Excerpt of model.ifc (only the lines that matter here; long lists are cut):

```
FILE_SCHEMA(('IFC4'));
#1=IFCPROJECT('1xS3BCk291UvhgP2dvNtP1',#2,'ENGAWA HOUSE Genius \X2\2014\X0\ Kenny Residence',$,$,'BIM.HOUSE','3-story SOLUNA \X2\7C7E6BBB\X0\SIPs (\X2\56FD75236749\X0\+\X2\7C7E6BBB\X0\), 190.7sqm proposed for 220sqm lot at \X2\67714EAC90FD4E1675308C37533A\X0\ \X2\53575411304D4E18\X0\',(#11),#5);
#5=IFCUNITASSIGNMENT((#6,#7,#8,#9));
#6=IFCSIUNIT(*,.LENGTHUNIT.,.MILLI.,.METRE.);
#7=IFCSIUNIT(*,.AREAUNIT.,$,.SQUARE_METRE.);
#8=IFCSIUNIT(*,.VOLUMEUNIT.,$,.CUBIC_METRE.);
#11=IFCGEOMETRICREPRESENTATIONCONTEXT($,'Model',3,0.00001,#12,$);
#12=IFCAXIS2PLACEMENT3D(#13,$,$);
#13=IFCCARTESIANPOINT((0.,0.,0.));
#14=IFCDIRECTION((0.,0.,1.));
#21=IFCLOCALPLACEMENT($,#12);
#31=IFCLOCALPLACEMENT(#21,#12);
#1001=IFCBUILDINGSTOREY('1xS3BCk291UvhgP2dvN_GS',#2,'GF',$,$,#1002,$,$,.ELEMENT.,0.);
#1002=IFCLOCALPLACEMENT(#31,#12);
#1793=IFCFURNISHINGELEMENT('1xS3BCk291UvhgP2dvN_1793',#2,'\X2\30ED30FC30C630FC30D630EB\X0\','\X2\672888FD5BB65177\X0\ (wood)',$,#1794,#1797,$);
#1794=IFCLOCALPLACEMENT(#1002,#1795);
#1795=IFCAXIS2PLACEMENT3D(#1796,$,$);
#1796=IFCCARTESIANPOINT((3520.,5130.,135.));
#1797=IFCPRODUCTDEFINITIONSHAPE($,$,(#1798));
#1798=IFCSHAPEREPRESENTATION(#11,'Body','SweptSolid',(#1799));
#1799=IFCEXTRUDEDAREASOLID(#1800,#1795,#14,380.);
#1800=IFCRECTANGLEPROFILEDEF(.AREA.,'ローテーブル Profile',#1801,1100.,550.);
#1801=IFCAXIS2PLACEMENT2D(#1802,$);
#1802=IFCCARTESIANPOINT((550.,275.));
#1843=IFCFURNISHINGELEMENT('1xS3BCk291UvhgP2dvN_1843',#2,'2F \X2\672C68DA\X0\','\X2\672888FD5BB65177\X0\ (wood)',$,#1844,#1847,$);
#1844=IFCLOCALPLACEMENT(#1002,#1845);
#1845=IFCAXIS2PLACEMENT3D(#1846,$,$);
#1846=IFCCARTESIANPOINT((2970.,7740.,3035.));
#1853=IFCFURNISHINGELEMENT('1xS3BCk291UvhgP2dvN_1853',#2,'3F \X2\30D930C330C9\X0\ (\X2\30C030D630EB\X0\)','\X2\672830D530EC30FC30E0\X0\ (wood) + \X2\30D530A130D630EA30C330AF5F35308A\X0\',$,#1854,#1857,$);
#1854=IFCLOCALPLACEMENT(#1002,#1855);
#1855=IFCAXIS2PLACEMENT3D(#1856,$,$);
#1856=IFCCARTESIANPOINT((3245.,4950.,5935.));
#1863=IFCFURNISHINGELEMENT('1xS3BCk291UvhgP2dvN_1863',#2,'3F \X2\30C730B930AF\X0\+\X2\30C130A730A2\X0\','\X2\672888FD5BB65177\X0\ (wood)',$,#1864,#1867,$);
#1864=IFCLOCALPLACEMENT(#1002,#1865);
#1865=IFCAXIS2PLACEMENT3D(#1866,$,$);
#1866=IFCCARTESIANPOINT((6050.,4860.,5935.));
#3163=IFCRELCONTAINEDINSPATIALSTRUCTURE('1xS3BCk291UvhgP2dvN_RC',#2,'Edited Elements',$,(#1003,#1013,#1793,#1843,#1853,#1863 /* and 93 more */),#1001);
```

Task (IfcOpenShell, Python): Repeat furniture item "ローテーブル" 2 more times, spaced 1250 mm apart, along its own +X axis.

```python
import ifcopenshell
import ifcopenshell.api.geometry
import ifcopenshell.api.root
import ifcopenshell.util.element
import ifcopenshell.util.placement
import ifcopenshell.util.unit

model = ifcopenshell.open("model.ifc")
unit_scale = ifcopenshell.util.unit.calculate_unit_scale(model)


def reuse_history(source, copy):
    """copy_class also copies each property set's owner history, people and application; keep the originals."""
    for rel in copy.IsDefinedBy:
        if rel.is_a("IfcRelDefinesByProperties") and (history := rel.RelatingPropertyDefinition.OwnerHistory):
            rel.RelatingPropertyDefinition.OwnerHistory = source.OwnerHistory
            ifcopenshell.util.element.remove_deep2(model, history)


source = model.by_id(1793)
base = ifcopenshell.util.placement.get_local_placement(source.ObjectPlacement)
step = base[:3, 0] * 1.25 / unit_scale

for i in range(1, 3):
    copy = ifcopenshell.api.root.copy_class(model, product=source)
    copy.Representation = ifcopenshell.util.element.copy_deep(
        model, source.Representation, exclude=["IfcGeometricRepresentationContext", "IfcRepresentationMap"]
    )
    reuse_history(source, copy)
    matrix = base.copy()
    matrix[:3, 3] += i * step
    print("added at", matrix[:3, 3].round(3) + 0.0)
    ifcopenshell.api.geometry.edit_object_placement(model, product=copy, matrix=matrix, is_si=False)

model.write("model-out.ifc")
```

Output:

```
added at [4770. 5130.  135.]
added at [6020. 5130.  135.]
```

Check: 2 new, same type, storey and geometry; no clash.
